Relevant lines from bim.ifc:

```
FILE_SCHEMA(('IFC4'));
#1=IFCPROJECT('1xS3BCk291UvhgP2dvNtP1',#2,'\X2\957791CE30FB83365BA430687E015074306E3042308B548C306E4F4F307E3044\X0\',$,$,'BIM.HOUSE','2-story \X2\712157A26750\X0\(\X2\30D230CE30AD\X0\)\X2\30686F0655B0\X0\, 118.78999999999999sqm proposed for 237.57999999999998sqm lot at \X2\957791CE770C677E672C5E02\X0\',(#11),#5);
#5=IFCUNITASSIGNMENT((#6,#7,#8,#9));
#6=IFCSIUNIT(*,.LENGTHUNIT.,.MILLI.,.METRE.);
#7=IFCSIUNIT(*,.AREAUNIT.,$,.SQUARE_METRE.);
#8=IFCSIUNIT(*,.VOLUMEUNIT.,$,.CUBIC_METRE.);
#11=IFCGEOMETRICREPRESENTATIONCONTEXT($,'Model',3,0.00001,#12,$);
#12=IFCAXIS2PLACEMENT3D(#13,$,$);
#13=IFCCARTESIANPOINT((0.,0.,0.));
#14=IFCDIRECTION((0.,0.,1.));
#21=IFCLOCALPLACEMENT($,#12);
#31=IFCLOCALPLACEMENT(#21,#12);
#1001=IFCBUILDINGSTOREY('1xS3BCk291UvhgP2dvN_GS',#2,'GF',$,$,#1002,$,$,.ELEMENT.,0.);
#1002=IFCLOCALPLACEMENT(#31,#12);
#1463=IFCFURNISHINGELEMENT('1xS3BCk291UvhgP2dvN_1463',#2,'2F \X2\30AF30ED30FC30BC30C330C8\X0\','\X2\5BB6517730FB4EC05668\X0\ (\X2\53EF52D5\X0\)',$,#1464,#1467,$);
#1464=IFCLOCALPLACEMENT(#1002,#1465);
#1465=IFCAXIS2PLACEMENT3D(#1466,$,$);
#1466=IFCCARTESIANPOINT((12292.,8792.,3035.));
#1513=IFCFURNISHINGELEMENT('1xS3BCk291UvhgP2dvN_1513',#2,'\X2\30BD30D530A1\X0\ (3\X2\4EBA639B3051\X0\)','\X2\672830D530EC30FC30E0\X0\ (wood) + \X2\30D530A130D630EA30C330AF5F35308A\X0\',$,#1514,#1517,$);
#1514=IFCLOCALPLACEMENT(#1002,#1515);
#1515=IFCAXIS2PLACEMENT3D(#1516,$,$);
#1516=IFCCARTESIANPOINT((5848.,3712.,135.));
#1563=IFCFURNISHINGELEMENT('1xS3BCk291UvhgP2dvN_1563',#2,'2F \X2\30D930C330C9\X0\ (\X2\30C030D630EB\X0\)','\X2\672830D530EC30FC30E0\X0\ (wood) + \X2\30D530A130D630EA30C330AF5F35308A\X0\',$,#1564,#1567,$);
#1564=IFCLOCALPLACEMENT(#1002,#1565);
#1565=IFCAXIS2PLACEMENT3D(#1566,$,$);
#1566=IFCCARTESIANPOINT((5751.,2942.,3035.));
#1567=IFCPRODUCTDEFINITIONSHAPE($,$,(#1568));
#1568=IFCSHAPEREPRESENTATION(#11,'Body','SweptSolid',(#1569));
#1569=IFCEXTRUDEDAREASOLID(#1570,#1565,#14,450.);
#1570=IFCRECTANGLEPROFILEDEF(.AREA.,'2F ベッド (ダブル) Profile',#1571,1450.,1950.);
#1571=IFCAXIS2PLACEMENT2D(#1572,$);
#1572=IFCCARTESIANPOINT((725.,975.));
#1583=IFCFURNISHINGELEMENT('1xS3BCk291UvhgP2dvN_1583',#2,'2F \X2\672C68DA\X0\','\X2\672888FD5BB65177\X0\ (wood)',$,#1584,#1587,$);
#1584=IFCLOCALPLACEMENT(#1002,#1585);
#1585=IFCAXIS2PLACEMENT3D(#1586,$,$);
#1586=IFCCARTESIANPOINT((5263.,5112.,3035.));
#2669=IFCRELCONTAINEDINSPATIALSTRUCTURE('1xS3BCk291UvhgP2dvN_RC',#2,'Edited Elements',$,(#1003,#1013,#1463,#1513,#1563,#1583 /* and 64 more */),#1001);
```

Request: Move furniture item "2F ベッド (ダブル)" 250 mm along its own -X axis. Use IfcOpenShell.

```python
import ifcopenshell
import ifcopenshell.api.geometry
import ifcopenshell.util.placement

model = ifcopenshell.open("bim.ifc")

item = model.by_guid("1xS3BCk291UvhgP2dvN_1563")
matrix = ifcopenshell.util.placement.get_local_placement(item.ObjectPlacement)
matrix[:3, 3] -= matrix[:3, 0] * 250.0
ifcopenshell.api.geometry.edit_object_placement(model, product=item, matrix=matrix, is_si=False)

print(ifcopenshell.util.placement.get_local_placement(item.ObjectPlacement).round(3) + 0.0)

model.write("bim-out.ifc")
```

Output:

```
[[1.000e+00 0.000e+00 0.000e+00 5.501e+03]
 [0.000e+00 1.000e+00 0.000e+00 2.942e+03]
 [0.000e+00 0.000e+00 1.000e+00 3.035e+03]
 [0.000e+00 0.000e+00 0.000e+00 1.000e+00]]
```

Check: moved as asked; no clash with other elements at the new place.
